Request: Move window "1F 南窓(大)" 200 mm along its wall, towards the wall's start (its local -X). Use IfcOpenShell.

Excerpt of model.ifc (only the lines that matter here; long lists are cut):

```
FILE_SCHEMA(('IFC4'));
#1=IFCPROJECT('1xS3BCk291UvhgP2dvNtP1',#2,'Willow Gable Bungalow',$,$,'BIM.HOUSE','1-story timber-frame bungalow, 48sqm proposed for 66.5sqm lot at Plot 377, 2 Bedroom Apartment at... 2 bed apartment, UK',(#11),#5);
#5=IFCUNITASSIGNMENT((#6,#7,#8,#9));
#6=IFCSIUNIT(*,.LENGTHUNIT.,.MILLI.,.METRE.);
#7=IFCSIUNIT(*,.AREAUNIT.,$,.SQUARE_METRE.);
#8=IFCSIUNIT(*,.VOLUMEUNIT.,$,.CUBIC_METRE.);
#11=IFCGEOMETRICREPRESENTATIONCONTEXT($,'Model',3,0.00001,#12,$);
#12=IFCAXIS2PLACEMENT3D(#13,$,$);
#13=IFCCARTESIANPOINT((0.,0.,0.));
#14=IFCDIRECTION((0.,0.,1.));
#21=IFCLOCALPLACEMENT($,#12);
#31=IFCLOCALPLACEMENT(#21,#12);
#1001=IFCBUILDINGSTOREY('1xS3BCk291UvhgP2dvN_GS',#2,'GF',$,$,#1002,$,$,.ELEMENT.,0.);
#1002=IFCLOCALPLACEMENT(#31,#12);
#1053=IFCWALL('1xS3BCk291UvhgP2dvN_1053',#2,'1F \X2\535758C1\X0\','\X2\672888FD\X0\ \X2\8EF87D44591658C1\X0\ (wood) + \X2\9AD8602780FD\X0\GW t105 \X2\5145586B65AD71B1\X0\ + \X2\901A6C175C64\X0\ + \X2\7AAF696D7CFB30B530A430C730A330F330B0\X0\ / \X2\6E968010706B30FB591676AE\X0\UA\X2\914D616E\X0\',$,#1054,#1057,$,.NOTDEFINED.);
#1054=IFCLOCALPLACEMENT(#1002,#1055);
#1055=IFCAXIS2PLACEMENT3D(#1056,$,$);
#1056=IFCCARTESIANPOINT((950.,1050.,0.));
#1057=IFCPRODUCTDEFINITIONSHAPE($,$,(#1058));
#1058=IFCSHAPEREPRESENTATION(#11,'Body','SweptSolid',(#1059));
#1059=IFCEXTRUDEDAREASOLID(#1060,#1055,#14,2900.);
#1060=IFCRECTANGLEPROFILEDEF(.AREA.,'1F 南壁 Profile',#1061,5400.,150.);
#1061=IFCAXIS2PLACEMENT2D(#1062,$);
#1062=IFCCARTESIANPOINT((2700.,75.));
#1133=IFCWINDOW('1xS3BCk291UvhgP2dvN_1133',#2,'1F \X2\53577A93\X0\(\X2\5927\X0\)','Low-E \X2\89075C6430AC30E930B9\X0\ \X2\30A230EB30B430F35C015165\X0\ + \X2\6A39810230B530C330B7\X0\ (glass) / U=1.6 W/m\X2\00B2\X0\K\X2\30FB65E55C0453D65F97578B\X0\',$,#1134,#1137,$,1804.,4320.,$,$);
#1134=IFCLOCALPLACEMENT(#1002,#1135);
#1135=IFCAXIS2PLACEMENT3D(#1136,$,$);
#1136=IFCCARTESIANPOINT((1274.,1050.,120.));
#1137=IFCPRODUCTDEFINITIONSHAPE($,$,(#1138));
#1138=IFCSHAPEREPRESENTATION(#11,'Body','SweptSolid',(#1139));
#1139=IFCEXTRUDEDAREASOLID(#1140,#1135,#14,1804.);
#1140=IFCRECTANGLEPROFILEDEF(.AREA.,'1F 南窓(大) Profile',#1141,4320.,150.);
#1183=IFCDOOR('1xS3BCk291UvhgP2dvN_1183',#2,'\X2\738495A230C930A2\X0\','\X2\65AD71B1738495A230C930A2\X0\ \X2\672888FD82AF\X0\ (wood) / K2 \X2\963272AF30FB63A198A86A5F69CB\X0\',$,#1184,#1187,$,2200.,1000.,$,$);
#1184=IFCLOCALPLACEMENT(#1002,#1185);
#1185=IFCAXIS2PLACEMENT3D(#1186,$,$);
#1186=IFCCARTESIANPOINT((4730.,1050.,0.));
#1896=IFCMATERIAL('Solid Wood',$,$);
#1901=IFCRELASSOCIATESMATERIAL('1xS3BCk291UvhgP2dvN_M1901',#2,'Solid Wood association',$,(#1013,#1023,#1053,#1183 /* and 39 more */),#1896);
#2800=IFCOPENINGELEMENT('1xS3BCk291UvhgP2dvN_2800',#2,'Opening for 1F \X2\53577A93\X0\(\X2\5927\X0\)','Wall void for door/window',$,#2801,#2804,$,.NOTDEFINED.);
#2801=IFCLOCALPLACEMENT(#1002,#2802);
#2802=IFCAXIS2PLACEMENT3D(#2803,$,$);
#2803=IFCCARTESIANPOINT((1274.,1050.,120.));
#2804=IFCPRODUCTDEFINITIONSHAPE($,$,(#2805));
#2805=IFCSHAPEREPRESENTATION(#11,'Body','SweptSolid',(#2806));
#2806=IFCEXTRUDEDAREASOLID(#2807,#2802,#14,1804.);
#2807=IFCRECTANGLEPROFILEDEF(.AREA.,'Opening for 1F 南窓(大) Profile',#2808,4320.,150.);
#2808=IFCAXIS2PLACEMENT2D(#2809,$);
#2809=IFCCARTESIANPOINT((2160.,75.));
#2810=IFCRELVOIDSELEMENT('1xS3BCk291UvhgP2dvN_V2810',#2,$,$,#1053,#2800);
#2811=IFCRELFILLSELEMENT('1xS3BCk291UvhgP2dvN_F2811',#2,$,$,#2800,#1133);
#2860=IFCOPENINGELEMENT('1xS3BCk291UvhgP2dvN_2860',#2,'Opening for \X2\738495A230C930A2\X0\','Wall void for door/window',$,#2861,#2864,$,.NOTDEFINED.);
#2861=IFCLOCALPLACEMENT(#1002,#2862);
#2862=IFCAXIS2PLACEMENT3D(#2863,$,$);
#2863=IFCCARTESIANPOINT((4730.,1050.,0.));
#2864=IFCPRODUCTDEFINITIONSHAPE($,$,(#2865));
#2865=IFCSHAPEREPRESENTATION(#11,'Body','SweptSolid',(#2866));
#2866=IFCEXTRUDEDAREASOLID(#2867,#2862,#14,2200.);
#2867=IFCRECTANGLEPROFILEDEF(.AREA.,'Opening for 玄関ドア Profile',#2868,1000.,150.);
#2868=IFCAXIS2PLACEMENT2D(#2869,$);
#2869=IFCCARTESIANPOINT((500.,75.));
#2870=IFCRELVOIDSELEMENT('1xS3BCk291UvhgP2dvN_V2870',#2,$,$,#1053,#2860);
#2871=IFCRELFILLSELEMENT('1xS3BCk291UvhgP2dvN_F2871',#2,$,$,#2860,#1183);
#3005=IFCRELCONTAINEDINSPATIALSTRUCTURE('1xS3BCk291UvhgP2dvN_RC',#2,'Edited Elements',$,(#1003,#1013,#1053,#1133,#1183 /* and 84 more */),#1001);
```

```python
import ifcopenshell
import ifcopenshell.api.geometry
import ifcopenshell.util.placement

model = ifcopenshell.open("model.ifc")

window = model.by_id(1133)
opening = window.FillsVoids[0].RelatingOpeningElement
wall = opening.VoidsElements[0].RelatingBuildingElement

wall_matrix = ifcopenshell.util.placement.get_local_placement(wall.ObjectPlacement)
shift = wall_matrix[:3, 0] * -200.0
before = ifcopenshell.util.placement.get_local_placement(window.ObjectPlacement)[:3, 3].copy()

# The window is not placed relative to its opening, so move both.
for product in (opening, window):
    matrix = ifcopenshell.util.placement.get_local_placement(product.ObjectPlacement)
    matrix[:3, 3] += shift
    ifcopenshell.api.geometry.edit_object_placement(model, product=product, matrix=matrix, is_si=False)

after = ifcopenshell.util.placement.get_local_placement(window.ObjectPlacement)[:3, 3]
print("window moved by", (after - before).round(3) + 0.0)

model.write("model_updated.ifc")
```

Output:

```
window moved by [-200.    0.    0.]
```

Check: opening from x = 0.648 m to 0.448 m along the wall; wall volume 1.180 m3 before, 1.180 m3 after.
